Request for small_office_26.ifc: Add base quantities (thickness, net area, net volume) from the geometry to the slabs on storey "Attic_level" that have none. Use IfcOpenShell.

First a look at what the model holds.

```python
import ifcopenshell
import ifcopenshell.util.element
import ifcopenshell.util.unit

model = ifcopenshell.open("small_office_26.ifc")
print(model.schema)
for unit_type in ("LENGTHUNIT", "AREAUNIT", "VOLUMEUNIT"):
    print(unit_type, ifcopenshell.util.unit.calculate_unit_scale(model, unit_type))
storey = next(s for s in model.by_type("IfcBuildingStorey") if s.Name == "Attic_level")
slabs = [e for e in ifcopenshell.util.element.get_decomposition(storey) if e.is_a("IfcSlab")]
for e in sorted(slabs, key=lambda e: e.id()):
    print(e.id(), e.is_a(), e.Name, list(ifcopenshell.util.element.get_psets(e, qtos_only=True)), sep=" | ")
```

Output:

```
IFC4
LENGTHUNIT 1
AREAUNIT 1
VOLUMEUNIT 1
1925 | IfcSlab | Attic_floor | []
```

```python
import ifcopenshell
import ifcopenshell.api.pset
import ifcopenshell.geom
import ifcopenshell.util.element
import ifcopenshell.util.shape
import ifcopenshell.util.unit

model = ifcopenshell.open("small_office_26.ifc")
unit_scale = ifcopenshell.util.unit.calculate_unit_scale(model)
area_scale = ifcopenshell.util.unit.calculate_unit_scale(model, "AREAUNIT")
volume_scale = ifcopenshell.util.unit.calculate_unit_scale(model, "VOLUMEUNIT")
settings = ifcopenshell.geom.settings()

storey = next(s for s in model.by_type("IfcBuildingStorey") if s.Name == "Attic_level")
slabs = [e for e in ifcopenshell.util.element.get_decomposition(storey) if e.is_a("IfcSlab")]

for e in sorted(slabs, key=lambda e: e.id()):
    if ifcopenshell.util.element.get_psets(e, qtos_only=True, should_inherit=False):
        continue
    # Geometry comes back in metres, in the element's own axes.
    shape = ifcopenshell.geom.create_shape(settings, e)
    values = {
        "Width": ifcopenshell.util.shape.get_z(shape.geometry) / unit_scale,
        "NetArea": ifcopenshell.util.shape.get_footprint_area(shape.geometry) / area_scale,
        "NetVolume": ifcopenshell.util.shape.get_volume(shape.geometry) / volume_scale,
    }
    qto = ifcopenshell.api.pset.add_qto(model, product=e, name="Qto_SlabBaseQuantities")
    ifcopenshell.api.pset.edit_qto(model, qto=qto, properties=values)
    print(e.id(), {k: round(v, 3) for k, v in values.items()})

model.write("small_office_26-out.ifc")
```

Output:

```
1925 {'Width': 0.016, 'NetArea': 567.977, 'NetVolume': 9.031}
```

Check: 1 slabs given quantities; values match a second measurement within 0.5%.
